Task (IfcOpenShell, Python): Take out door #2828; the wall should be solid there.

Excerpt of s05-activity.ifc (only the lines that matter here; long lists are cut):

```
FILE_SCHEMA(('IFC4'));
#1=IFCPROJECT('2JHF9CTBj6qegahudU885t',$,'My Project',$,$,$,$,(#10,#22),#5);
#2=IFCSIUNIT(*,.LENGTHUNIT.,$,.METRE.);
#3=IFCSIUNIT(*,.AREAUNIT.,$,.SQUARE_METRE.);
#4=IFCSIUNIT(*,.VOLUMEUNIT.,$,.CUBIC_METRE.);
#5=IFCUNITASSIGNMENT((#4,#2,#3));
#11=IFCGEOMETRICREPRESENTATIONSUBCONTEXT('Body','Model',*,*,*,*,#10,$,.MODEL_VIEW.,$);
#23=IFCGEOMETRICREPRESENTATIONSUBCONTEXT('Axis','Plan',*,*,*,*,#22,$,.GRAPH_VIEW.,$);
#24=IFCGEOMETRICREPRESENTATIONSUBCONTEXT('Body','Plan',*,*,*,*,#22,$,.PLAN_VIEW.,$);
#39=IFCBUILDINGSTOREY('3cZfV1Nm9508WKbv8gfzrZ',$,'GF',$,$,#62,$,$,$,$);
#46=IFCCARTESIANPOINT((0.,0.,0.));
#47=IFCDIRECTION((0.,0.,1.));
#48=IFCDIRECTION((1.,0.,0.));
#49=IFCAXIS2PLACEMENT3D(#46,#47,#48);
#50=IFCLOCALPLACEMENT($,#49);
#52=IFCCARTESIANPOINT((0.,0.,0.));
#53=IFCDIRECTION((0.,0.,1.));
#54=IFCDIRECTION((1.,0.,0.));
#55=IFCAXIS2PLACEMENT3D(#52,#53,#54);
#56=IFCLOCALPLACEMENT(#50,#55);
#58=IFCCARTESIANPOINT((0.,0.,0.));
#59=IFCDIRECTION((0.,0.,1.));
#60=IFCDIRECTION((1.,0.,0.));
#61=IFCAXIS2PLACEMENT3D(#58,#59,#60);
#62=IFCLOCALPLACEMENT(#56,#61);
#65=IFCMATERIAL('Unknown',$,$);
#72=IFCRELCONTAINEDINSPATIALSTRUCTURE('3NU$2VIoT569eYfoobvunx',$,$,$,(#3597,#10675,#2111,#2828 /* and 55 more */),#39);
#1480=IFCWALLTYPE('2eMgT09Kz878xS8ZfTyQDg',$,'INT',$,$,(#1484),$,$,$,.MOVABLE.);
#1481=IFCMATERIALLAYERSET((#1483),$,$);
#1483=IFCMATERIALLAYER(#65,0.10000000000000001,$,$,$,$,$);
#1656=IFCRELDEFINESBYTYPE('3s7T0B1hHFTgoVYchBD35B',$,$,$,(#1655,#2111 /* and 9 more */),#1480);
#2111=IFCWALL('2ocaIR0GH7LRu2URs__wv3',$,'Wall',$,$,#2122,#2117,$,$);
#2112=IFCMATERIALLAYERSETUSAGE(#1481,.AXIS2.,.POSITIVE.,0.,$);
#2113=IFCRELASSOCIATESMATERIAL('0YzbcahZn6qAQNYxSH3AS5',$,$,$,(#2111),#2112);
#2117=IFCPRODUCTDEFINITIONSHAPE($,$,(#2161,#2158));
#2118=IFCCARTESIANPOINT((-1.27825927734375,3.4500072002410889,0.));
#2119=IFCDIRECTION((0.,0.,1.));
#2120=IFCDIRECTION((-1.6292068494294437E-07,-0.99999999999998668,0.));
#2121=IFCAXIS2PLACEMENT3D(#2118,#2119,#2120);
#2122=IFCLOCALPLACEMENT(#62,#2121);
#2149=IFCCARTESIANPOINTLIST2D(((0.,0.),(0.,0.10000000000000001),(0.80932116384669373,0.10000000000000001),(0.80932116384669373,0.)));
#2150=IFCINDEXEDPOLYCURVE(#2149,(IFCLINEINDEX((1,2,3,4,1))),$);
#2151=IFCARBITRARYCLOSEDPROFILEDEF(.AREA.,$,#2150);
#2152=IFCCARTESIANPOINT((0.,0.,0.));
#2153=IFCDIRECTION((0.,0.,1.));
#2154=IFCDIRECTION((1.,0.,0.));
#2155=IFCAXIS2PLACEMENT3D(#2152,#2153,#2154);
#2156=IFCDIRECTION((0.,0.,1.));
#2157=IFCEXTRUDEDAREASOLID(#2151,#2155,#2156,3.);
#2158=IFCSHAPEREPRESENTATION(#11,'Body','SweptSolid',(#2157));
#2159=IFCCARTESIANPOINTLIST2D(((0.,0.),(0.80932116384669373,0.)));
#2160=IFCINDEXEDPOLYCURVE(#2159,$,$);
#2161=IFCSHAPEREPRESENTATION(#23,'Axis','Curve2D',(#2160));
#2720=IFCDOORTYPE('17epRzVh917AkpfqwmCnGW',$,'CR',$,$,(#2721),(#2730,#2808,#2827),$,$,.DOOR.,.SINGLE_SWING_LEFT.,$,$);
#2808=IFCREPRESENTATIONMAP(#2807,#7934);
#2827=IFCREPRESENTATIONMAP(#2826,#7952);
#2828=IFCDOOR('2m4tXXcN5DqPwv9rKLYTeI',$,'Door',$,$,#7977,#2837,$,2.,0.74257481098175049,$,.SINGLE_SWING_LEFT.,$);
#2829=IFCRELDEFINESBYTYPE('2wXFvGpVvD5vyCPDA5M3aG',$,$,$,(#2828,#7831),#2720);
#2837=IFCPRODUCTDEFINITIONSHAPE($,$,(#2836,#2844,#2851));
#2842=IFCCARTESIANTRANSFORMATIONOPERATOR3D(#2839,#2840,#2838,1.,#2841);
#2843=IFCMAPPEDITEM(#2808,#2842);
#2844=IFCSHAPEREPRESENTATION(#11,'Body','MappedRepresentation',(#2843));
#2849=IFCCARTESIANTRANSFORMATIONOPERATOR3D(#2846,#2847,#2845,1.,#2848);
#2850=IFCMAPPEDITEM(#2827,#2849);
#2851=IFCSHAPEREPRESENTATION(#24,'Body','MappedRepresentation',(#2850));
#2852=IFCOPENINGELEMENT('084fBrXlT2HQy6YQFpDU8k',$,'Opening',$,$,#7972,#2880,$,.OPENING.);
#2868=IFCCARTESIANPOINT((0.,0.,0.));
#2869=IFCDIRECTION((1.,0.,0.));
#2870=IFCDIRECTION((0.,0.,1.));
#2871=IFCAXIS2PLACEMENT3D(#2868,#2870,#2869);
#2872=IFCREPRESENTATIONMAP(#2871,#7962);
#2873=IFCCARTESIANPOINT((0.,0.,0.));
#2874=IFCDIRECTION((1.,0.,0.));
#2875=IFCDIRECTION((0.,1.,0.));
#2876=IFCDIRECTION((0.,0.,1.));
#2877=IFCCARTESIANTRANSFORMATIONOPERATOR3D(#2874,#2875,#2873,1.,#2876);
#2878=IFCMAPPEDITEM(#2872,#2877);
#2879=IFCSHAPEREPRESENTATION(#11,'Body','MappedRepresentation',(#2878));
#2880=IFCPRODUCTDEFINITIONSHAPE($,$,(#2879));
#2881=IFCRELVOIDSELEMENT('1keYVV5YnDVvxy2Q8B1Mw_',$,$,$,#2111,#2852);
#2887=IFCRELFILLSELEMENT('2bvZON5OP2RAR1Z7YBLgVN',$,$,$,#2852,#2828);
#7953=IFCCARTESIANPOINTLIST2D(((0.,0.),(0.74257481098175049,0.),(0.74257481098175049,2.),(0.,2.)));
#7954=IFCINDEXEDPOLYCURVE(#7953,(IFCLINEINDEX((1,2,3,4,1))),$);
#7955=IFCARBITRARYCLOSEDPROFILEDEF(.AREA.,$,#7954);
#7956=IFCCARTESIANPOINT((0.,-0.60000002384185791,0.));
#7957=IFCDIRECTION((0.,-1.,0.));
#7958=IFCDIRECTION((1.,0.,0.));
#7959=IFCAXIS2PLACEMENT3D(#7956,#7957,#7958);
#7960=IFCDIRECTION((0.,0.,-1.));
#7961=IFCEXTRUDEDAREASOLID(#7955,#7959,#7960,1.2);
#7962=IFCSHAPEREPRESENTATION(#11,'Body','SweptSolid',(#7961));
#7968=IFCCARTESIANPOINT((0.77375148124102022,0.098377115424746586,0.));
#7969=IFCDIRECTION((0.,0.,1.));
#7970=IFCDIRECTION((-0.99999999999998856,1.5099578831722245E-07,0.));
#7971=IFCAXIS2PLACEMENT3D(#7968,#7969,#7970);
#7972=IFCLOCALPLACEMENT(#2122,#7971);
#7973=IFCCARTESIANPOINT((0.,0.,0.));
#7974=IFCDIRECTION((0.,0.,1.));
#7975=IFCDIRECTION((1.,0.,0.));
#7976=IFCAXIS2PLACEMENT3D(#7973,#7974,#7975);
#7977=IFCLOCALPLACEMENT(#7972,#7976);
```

```python
import ifcopenshell
import ifcopenshell.api.feature
import ifcopenshell.api.root
import ifcopenshell.geom
import ifcopenshell.util.shape

model = ifcopenshell.open("s05-activity.ifc")
settings = ifcopenshell.geom.settings()


def volume(element):
    """Net volume in cubic metres, openings subtracted."""
    shape = ifcopenshell.geom.create_shape(settings, element)
    return ifcopenshell.util.shape.get_volume(shape.geometry)


door = model.by_id(2828)
opening = door.FillsVoids[0].RelatingOpeningElement
wall = opening.VoidsElements[0].RelatingBuildingElement
before = volume(wall)

ifcopenshell.api.root.remove_product(model, product=door)
ifcopenshell.api.feature.remove_feature(model, feature=opening)

after = volume(wall)

print(f"wall volume {before:.3f} -> {after:.3f} m3")

model.write("s05-activity-out.ifc")
```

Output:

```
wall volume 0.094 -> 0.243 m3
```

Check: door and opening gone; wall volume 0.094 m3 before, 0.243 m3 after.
